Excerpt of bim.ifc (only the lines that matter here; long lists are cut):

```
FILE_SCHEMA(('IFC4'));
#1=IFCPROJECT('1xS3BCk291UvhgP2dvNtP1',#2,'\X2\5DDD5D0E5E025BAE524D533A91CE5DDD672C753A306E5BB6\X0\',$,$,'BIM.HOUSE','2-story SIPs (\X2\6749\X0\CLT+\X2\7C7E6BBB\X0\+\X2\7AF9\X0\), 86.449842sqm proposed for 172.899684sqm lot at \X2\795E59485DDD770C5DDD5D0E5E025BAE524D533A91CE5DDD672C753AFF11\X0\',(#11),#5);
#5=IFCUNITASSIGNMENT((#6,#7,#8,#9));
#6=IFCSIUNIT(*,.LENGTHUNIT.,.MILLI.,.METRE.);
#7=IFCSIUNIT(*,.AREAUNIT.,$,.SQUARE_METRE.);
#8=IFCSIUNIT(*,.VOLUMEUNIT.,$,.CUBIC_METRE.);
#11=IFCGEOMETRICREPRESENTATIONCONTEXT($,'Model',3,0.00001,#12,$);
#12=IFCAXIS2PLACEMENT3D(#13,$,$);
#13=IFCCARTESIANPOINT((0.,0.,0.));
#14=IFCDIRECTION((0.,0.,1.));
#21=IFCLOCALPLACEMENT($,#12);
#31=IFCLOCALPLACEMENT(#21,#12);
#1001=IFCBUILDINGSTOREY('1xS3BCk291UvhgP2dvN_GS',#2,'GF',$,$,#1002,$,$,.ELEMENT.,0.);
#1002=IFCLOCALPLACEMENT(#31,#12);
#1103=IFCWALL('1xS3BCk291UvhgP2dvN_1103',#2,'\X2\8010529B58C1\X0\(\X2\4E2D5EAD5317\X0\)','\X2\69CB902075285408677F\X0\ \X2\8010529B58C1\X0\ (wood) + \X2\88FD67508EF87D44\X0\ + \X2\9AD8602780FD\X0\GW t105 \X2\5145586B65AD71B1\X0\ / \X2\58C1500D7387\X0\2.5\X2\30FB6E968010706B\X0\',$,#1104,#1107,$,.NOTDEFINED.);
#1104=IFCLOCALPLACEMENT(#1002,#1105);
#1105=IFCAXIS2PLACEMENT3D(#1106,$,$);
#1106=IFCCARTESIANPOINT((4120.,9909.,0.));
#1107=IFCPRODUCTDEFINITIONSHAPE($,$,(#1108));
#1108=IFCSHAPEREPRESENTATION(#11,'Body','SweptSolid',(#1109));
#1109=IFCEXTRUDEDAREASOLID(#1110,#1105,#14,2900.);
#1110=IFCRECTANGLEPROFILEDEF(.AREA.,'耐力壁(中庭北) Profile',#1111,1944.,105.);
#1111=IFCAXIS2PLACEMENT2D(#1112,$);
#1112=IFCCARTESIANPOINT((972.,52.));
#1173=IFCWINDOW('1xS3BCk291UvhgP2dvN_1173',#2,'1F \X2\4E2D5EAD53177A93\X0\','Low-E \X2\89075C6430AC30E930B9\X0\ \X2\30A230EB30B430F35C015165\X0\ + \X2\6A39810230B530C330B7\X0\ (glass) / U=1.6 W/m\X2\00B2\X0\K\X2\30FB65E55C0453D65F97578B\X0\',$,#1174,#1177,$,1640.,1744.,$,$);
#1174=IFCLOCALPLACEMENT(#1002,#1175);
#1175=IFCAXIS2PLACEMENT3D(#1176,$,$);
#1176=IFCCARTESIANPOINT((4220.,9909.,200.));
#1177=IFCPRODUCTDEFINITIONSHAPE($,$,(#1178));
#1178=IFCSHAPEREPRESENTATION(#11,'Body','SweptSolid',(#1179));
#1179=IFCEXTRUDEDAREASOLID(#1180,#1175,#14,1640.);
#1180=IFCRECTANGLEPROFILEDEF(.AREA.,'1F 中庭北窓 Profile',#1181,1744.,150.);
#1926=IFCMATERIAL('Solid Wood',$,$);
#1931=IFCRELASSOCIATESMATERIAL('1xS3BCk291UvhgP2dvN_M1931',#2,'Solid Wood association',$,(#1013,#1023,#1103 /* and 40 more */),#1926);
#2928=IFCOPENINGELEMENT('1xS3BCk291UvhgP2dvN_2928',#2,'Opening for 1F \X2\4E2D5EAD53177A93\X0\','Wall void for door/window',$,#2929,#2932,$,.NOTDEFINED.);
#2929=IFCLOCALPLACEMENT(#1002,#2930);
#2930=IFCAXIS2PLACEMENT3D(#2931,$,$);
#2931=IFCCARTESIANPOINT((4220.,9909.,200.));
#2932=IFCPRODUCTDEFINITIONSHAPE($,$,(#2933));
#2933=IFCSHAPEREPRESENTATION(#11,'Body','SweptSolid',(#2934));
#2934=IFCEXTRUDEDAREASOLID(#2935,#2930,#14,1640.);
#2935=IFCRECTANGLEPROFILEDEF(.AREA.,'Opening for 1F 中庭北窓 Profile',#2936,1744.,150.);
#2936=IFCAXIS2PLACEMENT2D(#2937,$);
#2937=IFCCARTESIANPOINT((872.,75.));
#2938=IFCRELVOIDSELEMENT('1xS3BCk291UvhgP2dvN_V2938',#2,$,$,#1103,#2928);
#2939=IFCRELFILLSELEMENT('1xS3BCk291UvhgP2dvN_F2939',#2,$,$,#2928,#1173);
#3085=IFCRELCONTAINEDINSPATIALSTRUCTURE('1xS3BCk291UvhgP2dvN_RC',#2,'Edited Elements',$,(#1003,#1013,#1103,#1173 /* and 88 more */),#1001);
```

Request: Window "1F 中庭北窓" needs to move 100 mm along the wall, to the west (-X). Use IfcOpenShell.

```python
import ifcopenshell
import ifcopenshell.api.geometry
import ifcopenshell.util.placement

model = ifcopenshell.open("bim.ifc")

window = model.by_id(1173)
opening = window.FillsVoids[0].RelatingOpeningElement
wall = opening.VoidsElements[0].RelatingBuildingElement

wall_matrix = ifcopenshell.util.placement.get_local_placement(wall.ObjectPlacement)
shift = wall_matrix[:3, 0] * -100.0
before = ifcopenshell.util.placement.get_local_placement(window.ObjectPlacement)[:3, 3].copy()

# The window is not placed relative to its opening, so move both.
for product in (opening, window):
    matrix = ifcopenshell.util.placement.get_local_placement(product.ObjectPlacement)
    matrix[:3, 3] += shift
    ifcopenshell.api.geometry.edit_object_placement(model, product=product, matrix=matrix, is_si=False)

after = ifcopenshell.util.placement.get_local_placement(window.ObjectPlacement)[:3, 3]
print("window moved by", (after - before).round(3) + 0.0)

model.write("bim_updated.ifc")
```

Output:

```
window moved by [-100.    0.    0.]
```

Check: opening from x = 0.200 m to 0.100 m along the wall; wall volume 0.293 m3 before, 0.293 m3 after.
